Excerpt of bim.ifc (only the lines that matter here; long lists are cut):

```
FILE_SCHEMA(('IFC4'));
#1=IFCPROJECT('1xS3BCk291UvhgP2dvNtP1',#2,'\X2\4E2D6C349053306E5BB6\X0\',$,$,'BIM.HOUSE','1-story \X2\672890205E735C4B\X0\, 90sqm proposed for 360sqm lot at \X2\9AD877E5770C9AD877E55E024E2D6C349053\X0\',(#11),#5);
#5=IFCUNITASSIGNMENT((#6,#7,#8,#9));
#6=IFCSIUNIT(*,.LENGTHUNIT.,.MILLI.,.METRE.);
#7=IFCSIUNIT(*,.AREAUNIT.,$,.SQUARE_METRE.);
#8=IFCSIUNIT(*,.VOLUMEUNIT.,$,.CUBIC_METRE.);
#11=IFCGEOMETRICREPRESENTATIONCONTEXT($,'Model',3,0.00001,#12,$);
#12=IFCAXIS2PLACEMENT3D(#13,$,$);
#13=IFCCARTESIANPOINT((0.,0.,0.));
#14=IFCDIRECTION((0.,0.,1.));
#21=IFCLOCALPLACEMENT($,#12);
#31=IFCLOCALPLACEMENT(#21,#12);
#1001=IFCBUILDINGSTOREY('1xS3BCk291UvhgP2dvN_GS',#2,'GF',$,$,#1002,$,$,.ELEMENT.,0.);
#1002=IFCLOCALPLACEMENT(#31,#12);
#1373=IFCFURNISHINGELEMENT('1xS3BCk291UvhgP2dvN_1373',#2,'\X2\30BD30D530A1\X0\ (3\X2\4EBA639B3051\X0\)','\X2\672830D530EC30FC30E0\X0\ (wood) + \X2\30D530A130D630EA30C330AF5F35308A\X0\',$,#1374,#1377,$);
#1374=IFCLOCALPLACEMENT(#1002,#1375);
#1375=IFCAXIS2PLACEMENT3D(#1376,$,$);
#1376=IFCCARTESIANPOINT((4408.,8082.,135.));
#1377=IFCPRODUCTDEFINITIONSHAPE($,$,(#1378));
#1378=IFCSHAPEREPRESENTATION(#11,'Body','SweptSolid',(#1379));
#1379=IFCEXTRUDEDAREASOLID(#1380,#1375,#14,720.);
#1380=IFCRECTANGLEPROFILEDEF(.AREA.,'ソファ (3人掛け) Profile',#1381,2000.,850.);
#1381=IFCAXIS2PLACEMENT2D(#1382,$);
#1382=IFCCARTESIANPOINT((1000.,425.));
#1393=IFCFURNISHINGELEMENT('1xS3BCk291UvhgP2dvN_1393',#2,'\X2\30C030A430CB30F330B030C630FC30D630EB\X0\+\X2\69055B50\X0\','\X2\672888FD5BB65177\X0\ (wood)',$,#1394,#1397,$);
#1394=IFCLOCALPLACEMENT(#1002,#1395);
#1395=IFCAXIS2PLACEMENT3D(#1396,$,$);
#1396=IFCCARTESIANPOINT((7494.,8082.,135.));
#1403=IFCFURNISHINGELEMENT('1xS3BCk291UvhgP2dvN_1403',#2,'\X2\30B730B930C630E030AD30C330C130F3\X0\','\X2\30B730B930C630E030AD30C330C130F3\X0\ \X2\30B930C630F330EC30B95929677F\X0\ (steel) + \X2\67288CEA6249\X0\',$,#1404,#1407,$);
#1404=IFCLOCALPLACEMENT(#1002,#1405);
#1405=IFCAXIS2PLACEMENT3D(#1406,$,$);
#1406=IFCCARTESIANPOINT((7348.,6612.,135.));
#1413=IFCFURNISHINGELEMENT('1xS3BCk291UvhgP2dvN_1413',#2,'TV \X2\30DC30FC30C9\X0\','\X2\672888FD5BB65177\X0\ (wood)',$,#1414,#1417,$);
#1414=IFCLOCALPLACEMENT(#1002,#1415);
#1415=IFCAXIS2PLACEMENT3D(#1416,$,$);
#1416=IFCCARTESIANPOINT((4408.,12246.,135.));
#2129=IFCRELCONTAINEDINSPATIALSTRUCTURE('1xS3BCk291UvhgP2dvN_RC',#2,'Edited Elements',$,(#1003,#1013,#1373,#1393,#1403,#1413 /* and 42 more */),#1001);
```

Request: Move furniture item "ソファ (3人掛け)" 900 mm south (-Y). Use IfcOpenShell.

```python
import ifcopenshell
import ifcopenshell.api.geometry
import ifcopenshell.util.placement
import ifcopenshell.util.unit

model = ifcopenshell.open("bim.ifc")
unit_scale = ifcopenshell.util.unit.calculate_unit_scale(model)

item = model.by_guid("1xS3BCk291UvhgP2dvN_1373")
matrix = ifcopenshell.util.placement.get_local_placement(item.ObjectPlacement)
matrix[1, 3] -= 0.9 / unit_scale
ifcopenshell.api.geometry.edit_object_placement(model, product=item, matrix=matrix, is_si=False)

print(ifcopenshell.util.placement.get_local_placement(item.ObjectPlacement).round(3) + 0.0)

model.write("bim_rev.ifc")
```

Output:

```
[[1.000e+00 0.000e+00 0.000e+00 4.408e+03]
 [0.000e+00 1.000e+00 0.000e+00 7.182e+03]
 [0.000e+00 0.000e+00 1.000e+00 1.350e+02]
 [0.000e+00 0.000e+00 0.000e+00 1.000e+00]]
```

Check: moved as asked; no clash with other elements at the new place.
